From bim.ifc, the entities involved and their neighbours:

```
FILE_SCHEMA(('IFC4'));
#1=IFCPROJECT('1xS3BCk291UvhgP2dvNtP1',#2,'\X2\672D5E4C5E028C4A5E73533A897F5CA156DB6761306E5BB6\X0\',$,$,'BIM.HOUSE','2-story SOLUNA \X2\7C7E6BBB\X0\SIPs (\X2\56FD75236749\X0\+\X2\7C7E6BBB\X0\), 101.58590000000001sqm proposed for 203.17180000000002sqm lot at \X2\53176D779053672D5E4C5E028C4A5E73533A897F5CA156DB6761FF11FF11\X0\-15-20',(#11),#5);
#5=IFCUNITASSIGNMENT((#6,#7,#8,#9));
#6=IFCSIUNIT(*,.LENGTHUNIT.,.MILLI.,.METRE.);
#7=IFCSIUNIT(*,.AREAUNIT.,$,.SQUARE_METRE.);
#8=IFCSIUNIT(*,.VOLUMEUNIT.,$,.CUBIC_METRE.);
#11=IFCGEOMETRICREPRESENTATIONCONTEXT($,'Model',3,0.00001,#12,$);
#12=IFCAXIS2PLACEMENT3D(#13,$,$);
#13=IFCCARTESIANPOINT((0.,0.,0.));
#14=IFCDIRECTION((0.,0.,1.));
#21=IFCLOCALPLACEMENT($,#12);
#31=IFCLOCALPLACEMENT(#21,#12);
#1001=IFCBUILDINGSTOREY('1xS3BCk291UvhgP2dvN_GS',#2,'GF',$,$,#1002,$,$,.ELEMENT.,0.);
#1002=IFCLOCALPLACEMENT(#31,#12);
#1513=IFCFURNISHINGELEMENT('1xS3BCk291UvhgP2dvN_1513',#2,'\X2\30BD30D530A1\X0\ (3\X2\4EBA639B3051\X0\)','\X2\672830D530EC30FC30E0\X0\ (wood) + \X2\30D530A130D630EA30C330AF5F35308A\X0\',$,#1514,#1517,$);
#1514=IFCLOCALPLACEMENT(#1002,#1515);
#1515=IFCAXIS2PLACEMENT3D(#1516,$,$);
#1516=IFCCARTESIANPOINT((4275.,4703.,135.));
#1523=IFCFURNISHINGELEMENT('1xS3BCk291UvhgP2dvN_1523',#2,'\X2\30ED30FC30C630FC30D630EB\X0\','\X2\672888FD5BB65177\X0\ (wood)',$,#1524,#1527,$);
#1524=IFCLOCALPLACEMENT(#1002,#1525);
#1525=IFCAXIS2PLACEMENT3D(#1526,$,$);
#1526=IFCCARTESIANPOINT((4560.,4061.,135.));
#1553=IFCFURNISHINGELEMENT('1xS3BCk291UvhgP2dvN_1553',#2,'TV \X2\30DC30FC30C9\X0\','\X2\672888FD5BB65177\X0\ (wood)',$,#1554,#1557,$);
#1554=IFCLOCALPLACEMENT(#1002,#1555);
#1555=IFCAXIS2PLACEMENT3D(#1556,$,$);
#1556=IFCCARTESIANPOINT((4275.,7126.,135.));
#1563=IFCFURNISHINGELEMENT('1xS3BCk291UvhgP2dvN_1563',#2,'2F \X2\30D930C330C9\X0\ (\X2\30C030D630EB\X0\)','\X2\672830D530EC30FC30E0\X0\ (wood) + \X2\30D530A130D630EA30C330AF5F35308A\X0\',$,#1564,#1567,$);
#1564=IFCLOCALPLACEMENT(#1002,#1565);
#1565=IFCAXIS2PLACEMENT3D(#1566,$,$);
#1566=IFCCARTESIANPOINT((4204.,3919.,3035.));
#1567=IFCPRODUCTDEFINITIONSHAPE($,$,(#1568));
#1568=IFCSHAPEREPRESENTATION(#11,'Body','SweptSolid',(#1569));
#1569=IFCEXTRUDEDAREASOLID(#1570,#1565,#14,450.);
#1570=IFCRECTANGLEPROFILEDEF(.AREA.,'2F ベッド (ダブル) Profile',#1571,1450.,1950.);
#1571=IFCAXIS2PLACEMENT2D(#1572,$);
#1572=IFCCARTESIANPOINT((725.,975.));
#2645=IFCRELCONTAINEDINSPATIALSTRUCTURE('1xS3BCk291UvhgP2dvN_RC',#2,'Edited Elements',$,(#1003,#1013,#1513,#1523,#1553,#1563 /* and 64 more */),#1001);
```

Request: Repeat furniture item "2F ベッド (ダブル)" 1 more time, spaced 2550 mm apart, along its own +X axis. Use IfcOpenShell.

```python
import ifcopenshell
import ifcopenshell.api.geometry
import ifcopenshell.api.root
import ifcopenshell.util.element
import ifcopenshell.util.placement

model = ifcopenshell.open("bim.ifc")


def reuse_history(source, copy):
    """copy_class also copies each property set's owner history, people and application; keep the originals."""
    for rel in copy.IsDefinedBy:
        if rel.is_a("IfcRelDefinesByProperties") and (history := rel.RelatingPropertyDefinition.OwnerHistory):
            rel.RelatingPropertyDefinition.OwnerHistory = source.OwnerHistory
            ifcopenshell.util.element.remove_deep2(model, history)


source = model.by_guid("1xS3BCk291UvhgP2dvN_1563")
base = ifcopenshell.util.placement.get_local_placement(source.ObjectPlacement)
step = base[:3, 0] * 2550.0

for i in range(1, 2):
    copy = ifcopenshell.api.root.copy_class(model, product=source)
    copy.Representation = ifcopenshell.util.element.copy_deep(
        model, source.Representation, exclude=["IfcGeometricRepresentationContext", "IfcRepresentationMap"]
    )
    reuse_history(source, copy)
    matrix = base.copy()
    matrix[:3, 3] += i * step
    print("added at", matrix[:3, 3].round(3) + 0.0)
    ifcopenshell.api.geometry.edit_object_placement(model, product=copy, matrix=matrix, is_si=False)

model.write("bim_edited.ifc")
```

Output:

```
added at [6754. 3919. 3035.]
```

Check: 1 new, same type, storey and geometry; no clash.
